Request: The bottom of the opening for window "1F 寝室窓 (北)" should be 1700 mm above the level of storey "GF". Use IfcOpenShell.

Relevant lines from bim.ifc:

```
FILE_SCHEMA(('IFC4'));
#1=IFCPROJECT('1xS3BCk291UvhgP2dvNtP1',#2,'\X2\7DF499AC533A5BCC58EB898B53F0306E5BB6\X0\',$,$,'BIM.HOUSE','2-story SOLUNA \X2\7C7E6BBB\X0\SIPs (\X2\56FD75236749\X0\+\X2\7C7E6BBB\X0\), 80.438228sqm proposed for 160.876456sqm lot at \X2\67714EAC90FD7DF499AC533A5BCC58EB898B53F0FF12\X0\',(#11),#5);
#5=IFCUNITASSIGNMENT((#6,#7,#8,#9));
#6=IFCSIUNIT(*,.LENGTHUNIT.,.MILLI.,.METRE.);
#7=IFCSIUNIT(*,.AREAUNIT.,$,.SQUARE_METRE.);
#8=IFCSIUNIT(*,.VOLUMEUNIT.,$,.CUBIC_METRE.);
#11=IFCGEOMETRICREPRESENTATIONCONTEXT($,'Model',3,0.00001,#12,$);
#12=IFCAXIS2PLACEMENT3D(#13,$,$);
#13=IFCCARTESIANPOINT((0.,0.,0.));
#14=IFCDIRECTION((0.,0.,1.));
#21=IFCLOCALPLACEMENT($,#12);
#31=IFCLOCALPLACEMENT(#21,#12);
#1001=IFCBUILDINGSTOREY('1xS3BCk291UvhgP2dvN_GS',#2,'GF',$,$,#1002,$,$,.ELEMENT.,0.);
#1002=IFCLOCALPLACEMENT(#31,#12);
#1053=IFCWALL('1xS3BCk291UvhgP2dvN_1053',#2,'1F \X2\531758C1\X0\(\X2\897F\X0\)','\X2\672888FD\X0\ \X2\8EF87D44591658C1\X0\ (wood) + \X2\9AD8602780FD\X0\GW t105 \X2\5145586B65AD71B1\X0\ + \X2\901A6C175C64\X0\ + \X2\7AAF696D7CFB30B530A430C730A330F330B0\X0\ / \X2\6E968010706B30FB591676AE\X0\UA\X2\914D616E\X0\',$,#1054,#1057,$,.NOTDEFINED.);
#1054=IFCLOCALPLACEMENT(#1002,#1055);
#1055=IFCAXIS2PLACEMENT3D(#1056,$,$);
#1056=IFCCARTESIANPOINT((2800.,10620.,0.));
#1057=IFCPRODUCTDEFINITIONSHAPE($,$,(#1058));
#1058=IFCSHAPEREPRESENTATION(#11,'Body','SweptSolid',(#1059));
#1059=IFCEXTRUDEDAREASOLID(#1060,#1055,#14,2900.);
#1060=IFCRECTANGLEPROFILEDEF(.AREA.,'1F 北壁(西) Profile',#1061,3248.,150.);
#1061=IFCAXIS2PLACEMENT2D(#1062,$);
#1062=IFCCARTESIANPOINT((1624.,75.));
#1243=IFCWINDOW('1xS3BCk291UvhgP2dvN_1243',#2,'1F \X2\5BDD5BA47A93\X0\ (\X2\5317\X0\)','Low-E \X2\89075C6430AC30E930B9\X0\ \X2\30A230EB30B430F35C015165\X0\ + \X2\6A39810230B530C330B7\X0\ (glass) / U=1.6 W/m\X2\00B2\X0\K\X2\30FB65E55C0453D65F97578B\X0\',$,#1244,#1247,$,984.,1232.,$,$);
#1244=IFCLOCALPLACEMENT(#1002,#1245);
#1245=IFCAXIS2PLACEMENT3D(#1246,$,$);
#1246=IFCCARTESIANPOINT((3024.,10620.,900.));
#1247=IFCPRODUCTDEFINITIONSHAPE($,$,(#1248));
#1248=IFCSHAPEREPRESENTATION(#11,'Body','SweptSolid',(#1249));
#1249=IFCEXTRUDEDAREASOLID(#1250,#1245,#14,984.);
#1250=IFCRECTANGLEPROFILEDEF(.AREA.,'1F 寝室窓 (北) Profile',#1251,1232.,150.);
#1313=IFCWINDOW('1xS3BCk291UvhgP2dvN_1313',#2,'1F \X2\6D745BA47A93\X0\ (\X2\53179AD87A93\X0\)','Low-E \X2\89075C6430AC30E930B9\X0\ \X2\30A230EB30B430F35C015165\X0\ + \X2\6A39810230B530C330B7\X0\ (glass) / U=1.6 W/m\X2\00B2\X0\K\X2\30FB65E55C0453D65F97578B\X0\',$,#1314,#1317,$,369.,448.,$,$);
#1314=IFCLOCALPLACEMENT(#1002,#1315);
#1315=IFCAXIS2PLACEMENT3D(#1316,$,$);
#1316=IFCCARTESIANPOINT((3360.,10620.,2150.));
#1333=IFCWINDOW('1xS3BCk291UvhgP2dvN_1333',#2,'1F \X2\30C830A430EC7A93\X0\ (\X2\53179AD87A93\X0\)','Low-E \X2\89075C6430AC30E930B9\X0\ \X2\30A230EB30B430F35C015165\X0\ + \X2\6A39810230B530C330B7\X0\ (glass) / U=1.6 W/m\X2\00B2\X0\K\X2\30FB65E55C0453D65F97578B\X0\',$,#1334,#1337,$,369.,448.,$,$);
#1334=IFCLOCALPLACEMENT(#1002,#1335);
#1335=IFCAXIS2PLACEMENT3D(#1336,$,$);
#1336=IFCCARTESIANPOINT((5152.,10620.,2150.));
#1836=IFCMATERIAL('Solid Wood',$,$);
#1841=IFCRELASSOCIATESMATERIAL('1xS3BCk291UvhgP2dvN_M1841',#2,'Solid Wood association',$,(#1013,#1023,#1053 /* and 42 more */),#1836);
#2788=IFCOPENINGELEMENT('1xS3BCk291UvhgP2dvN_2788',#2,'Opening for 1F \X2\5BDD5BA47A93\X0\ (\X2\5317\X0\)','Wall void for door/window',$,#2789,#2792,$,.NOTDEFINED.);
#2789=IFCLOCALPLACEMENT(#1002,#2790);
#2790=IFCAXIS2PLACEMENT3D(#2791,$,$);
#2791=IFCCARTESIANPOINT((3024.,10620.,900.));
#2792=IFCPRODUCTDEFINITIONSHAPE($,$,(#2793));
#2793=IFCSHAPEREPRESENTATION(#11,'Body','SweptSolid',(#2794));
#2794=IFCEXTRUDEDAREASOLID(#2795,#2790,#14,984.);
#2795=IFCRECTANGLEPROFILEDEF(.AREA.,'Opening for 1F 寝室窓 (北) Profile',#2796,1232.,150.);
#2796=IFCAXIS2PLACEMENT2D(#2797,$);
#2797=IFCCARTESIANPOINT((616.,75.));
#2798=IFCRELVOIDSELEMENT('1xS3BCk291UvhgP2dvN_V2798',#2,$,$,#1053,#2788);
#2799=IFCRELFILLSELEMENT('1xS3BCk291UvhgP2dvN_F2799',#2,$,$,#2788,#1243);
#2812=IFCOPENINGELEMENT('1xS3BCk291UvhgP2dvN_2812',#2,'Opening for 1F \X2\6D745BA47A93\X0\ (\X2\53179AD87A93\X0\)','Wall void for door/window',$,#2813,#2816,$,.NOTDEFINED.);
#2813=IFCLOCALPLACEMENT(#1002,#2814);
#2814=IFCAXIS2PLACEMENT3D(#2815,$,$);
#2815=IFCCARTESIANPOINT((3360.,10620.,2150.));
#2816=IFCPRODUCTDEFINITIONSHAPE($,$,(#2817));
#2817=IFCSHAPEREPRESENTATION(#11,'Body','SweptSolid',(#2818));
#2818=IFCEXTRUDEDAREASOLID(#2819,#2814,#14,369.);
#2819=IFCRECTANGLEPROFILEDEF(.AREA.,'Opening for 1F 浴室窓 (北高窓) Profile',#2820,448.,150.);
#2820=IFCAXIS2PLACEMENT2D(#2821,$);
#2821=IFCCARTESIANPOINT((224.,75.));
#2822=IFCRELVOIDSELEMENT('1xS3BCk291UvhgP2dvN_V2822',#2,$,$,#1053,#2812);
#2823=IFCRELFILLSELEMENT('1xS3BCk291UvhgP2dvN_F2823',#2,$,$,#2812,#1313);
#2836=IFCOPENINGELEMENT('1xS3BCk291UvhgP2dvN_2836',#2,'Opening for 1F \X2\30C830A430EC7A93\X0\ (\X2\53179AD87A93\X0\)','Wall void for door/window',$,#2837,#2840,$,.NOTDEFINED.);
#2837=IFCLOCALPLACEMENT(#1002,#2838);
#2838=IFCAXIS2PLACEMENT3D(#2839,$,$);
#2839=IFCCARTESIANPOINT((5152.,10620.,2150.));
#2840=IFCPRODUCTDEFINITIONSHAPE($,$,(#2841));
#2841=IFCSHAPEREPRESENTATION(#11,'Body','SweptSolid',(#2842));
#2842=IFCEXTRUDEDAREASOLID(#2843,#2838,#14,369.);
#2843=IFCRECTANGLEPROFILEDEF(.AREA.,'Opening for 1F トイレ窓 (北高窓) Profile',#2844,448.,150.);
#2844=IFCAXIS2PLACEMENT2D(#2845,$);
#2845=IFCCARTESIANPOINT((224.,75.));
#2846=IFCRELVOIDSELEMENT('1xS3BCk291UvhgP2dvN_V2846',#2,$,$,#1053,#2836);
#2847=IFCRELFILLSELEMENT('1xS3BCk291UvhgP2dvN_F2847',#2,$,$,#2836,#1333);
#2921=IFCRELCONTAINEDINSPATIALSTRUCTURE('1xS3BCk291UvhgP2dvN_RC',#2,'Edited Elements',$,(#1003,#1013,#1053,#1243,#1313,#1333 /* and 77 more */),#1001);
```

```python
import numpy as np
import ifcopenshell
import ifcopenshell.api.geometry
import ifcopenshell.geom
import ifcopenshell.util.element
import ifcopenshell.util.placement
import ifcopenshell.util.shape
import ifcopenshell.util.unit

model = ifcopenshell.open("bim.ifc")
unit_scale = ifcopenshell.util.unit.calculate_unit_scale(model)

window = model.by_id(1243)
opening = window.FillsVoids[0].RelatingOpeningElement
storey = ifcopenshell.util.element.get_container(window, ifc_class="IfcBuildingStorey")
level = ifcopenshell.util.placement.get_local_placement(storey.ObjectPlacement)[2, 3]

# The opening's origin need not be at the sill, so measure its lowest point.
shape = ifcopenshell.geom.create_shape(ifcopenshell.geom.settings(), opening)
bottom = ifcopenshell.util.shape.get_shape_bottom_elevation(shape, shape.geometry) / unit_scale
dz = level + 1.7 / unit_scale - bottom

shift = np.array([0.0, 0.0, dz])
# The window is not placed relative to its opening, so move both.
for product in (opening, window):
    matrix = ifcopenshell.util.placement.get_local_placement(product.ObjectPlacement)
    matrix[:3, 3] += shift
    ifcopenshell.api.geometry.edit_object_placement(model, product=product, matrix=matrix, is_si=False)

print(f"moved by {dz * unit_scale:+.3f} m")

model.write("bim_updated.ifc")
```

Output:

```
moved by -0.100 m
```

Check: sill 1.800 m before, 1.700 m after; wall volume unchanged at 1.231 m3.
